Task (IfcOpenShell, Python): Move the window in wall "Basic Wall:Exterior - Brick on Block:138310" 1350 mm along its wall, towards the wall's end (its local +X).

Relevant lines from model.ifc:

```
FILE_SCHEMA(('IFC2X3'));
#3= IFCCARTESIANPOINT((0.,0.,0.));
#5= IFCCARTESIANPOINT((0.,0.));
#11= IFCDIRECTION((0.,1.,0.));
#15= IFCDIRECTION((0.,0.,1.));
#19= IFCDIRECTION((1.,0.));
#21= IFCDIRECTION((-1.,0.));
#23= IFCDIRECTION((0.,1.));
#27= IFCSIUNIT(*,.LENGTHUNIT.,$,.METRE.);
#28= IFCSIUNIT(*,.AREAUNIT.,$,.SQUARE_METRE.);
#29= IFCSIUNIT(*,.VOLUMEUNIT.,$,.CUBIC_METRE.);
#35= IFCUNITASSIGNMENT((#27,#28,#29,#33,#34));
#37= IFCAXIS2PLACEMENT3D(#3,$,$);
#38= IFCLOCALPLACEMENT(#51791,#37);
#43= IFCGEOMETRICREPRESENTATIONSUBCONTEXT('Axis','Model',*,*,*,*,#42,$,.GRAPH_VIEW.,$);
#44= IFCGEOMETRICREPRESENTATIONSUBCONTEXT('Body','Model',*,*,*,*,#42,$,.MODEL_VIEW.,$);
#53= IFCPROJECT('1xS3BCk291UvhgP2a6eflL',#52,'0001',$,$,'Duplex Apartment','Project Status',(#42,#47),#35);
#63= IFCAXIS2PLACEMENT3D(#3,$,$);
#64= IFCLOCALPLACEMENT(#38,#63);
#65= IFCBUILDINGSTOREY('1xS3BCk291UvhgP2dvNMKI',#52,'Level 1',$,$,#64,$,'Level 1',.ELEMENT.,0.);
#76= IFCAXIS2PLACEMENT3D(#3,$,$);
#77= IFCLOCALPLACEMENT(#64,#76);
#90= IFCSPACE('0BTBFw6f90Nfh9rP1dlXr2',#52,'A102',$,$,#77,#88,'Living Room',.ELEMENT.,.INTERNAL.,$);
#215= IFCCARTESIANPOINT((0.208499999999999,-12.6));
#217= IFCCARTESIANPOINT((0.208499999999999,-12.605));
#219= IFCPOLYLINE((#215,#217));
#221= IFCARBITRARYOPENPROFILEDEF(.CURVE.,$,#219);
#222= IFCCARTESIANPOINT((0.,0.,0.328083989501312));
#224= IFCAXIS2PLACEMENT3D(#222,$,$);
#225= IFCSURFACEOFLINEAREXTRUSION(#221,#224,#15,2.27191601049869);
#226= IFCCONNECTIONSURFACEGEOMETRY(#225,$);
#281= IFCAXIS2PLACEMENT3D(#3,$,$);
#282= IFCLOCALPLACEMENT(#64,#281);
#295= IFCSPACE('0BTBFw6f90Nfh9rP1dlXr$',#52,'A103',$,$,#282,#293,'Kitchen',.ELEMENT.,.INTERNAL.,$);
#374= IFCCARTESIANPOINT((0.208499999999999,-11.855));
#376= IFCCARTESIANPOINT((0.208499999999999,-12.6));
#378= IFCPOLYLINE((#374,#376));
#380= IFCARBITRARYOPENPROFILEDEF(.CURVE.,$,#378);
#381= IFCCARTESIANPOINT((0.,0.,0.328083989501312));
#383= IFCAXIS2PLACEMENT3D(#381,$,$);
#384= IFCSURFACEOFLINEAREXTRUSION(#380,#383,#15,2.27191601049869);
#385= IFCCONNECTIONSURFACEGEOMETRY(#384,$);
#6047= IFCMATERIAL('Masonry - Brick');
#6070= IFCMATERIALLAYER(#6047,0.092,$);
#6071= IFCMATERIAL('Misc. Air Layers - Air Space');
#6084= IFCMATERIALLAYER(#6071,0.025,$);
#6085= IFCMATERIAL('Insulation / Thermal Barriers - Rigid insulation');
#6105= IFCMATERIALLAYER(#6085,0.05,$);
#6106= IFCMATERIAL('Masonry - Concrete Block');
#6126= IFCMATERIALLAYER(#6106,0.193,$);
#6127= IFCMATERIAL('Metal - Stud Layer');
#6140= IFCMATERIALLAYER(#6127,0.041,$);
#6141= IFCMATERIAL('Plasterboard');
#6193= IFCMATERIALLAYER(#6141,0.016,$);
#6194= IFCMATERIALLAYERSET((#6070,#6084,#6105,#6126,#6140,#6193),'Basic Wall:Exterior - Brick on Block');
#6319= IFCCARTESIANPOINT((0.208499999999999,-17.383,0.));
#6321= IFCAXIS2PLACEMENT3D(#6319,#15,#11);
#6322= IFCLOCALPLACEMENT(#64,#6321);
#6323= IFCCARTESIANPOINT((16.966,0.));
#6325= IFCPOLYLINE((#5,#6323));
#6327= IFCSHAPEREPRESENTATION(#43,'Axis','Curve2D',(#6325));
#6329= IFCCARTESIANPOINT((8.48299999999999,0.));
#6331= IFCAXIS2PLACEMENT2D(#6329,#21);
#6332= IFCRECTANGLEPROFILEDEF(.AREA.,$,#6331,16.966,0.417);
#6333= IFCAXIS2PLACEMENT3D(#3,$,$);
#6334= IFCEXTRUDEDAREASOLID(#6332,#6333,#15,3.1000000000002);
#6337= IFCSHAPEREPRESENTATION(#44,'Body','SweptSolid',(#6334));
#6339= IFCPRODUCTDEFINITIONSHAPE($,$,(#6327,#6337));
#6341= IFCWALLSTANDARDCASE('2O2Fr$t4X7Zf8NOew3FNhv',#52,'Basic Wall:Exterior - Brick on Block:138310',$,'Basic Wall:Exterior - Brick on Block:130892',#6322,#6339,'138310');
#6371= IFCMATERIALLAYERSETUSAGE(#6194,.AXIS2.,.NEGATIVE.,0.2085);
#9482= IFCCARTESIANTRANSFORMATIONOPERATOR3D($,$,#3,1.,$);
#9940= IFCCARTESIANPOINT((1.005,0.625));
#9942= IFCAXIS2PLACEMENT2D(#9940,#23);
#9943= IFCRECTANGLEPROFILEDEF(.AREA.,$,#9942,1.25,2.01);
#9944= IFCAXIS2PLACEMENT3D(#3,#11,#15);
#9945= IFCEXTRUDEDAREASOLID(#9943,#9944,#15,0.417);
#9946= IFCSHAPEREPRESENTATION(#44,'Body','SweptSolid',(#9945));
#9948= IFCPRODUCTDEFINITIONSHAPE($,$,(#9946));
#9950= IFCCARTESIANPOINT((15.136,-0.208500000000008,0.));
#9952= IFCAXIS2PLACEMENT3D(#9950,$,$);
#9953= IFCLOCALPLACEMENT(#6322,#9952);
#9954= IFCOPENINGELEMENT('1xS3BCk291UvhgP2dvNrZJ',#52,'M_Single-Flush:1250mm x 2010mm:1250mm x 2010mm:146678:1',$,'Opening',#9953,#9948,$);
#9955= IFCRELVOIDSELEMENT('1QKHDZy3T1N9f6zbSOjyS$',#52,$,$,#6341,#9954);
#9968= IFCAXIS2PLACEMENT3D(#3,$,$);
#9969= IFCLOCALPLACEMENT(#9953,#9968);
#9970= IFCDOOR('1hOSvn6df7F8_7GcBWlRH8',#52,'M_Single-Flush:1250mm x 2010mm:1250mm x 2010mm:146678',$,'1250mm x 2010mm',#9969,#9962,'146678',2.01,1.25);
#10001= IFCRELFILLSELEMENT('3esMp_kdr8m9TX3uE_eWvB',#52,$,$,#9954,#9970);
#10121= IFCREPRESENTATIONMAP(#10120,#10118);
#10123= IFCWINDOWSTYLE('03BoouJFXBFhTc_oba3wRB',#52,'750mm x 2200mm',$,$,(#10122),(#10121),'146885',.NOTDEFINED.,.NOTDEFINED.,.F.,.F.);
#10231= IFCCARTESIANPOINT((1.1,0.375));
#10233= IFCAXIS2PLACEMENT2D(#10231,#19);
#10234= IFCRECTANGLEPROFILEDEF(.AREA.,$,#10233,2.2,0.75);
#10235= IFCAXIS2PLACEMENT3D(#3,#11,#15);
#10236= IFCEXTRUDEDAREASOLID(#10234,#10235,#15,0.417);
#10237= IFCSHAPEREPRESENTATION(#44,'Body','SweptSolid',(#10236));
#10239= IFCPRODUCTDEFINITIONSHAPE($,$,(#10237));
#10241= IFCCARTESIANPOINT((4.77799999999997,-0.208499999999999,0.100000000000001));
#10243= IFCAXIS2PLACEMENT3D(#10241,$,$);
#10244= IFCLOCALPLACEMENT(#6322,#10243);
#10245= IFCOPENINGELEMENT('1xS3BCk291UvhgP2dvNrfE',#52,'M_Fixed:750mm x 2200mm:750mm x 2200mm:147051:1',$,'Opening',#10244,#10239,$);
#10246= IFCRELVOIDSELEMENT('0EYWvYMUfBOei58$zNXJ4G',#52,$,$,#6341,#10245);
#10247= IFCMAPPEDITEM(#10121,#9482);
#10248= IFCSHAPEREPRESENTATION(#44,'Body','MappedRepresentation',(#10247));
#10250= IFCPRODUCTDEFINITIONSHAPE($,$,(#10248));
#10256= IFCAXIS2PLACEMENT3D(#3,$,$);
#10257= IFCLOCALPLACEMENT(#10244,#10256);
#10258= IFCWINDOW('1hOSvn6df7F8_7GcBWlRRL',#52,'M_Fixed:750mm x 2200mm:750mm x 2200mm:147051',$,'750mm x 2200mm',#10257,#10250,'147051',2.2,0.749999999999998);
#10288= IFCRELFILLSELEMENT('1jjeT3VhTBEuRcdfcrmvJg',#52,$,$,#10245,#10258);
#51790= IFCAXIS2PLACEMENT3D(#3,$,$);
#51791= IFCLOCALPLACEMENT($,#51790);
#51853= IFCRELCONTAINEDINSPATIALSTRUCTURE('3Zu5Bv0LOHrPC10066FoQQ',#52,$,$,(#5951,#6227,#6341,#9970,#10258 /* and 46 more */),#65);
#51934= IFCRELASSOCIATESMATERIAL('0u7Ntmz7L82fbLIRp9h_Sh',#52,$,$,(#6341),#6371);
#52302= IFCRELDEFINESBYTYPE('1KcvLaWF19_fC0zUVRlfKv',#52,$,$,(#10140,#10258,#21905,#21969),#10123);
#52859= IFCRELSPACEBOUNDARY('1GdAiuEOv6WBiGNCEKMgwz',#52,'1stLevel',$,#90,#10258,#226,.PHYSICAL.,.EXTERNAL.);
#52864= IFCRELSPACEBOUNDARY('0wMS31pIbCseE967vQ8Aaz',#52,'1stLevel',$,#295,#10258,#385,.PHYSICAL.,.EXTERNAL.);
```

```python
import numpy as np
import ifcopenshell
import ifcopenshell.api.geometry
import ifcopenshell.util.placement
import ifcopenshell.util.unit

model = ifcopenshell.open("model.ifc")
unit_scale = ifcopenshell.util.unit.calculate_unit_scale(model)

window = model.by_guid("1hOSvn6df7F8_7GcBWlRRL")
opening = window.FillsVoids[0].RelatingOpeningElement
wall = opening.VoidsElements[0].RelatingBuildingElement

wall_matrix = ifcopenshell.util.placement.get_local_placement(wall.ObjectPlacement)
shift = wall_matrix[:3, 0] * 1.35 / unit_scale
before = ifcopenshell.util.placement.get_local_placement(window.ObjectPlacement)[:3, 3].copy()

# The window is placed relative to its opening, so it follows when the opening moves.
matrix = ifcopenshell.util.placement.get_local_placement(opening.ObjectPlacement)
matrix[:3, 3] += shift
ifcopenshell.api.geometry.edit_object_placement(
    model, product=opening, matrix=matrix, is_si=False, should_transform_children=True
)

# Space boundary surfaces are stored in each space's coordinates; move them too.
for rel in window.ProvidesBoundaries:
    if not rel.ConnectionGeometry:
        continue
    surface = rel.ConnectionGeometry.SurfaceOnRelatingElement
    space_matrix = ifcopenshell.util.placement.get_local_placement(rel.RelatingSpace.ObjectPlacement)
    point = np.array(surface.Position.Location.Coordinates) + space_matrix[:3, :3].T @ shift
    surface.Position = model.createIfcAxis2Placement3D(
        model.createIfcCartesianPoint(point.tolist()), surface.Position.Axis, surface.Position.RefDirection
    )

after = ifcopenshell.util.placement.get_local_placement(window.ObjectPlacement)[:3, 3]
print("window moved by", (after - before).round(3) + 0.0)

model.write("model_v2.ifc")
```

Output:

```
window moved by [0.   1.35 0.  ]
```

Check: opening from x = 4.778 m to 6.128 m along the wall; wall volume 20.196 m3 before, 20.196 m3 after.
